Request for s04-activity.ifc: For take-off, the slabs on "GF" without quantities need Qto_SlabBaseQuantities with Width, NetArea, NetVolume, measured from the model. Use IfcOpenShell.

First a look at what the model holds.

```python
import ifcopenshell
import ifcopenshell.util.element
import ifcopenshell.util.unit

model = ifcopenshell.open("s04-activity.ifc")
print(model.schema)
for unit_type in ("LENGTHUNIT", "AREAUNIT", "VOLUMEUNIT"):
    print(unit_type, ifcopenshell.util.unit.calculate_unit_scale(model, unit_type))
storey = next(s for s in model.by_type("IfcBuildingStorey") if s.Name == "GF")
slabs = [e for e in ifcopenshell.util.element.get_decomposition(storey) if e.is_a("IfcSlab")]
for e in sorted(slabs, key=lambda e: e.id()):
    print(e.id(), e.is_a(), e.Name, list(ifcopenshell.util.element.get_psets(e, qtos_only=True)), sep=" | ")
```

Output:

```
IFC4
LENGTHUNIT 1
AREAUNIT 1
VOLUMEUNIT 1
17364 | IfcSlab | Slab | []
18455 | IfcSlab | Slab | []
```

```python
import ifcopenshell
import ifcopenshell.api.pset
import ifcopenshell.geom
import ifcopenshell.util.element
import ifcopenshell.util.shape
import ifcopenshell.util.unit

model = ifcopenshell.open("s04-activity.ifc")
unit_scale = ifcopenshell.util.unit.calculate_unit_scale(model)
area_scale = ifcopenshell.util.unit.calculate_unit_scale(model, "AREAUNIT")
volume_scale = ifcopenshell.util.unit.calculate_unit_scale(model, "VOLUMEUNIT")
settings = ifcopenshell.geom.settings()

storey = next(s for s in model.by_type("IfcBuildingStorey") if s.Name == "GF")
slabs = [e for e in ifcopenshell.util.element.get_decomposition(storey) if e.is_a("IfcSlab")]

for e in sorted(slabs, key=lambda e: e.id()):
    if ifcopenshell.util.element.get_psets(e, qtos_only=True, should_inherit=False):
        continue
    # Geometry comes back in metres, in the element's own axes.
    shape = ifcopenshell.geom.create_shape(settings, e)
    values = {
        "Width": ifcopenshell.util.shape.get_z(shape.geometry) / unit_scale,
        "NetArea": ifcopenshell.util.shape.get_footprint_area(shape.geometry) / area_scale,
        "NetVolume": ifcopenshell.util.shape.get_volume(shape.geometry) / volume_scale,
    }
    qto = ifcopenshell.api.pset.add_qto(model, product=e, name="Qto_SlabBaseQuantities")
    ifcopenshell.api.pset.edit_qto(model, qto=qto, properties=values)
    print(e.id(), {k: round(v, 3) for k, v in values.items()})

model.write("s04-activity-out.ifc")
```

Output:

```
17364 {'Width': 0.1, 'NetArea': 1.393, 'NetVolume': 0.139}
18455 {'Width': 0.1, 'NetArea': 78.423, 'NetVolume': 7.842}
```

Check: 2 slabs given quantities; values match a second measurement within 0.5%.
